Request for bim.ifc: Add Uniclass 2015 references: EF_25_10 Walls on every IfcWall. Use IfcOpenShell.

First a look at what the model holds.

```python
import ifcopenshell

model = ifcopenshell.open("bim.ifc")
print(model.schema)
print("classifications:", [c.Name for c in model.by_type("IfcClassification")])
for ifc_class in ("IfcDoor", "IfcRoof", "IfcStair", "IfcWall", "IfcWindow"):
    print(ifc_class, len(model.by_type(ifc_class)))
```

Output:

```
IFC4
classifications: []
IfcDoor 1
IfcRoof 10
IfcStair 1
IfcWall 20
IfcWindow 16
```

```python
import ifcopenshell
import ifcopenshell.api.classification

model = ifcopenshell.open("bim.ifc")

system = ifcopenshell.api.classification.add_classification(model, classification="Uniclass 2015")

codes = {
    "IfcWall": ("EF_25_10", "Walls"),
}
for ifc_class, (code, name) in codes.items():
    products = model.by_type(ifc_class)
    ifcopenshell.api.classification.add_reference(
        model, products=products, classification=system, identification=code, name=name
    )
    print(code, len(products))

model.write("bim_rev.ifc")
```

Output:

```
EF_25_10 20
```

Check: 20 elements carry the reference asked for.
